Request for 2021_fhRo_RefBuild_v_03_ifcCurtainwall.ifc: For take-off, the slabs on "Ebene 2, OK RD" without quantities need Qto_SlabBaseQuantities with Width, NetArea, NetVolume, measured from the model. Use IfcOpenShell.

First a look at what the model holds.

```python
import ifcopenshell
import ifcopenshell.util.element
import ifcopenshell.util.unit

model = ifcopenshell.open("2021_fhRo_RefBuild_v_03_ifcCurtainwall.ifc")
print(model.schema)
for unit_type in ("LENGTHUNIT", "AREAUNIT", "VOLUMEUNIT"):
    print(unit_type, ifcopenshell.util.unit.calculate_unit_scale(model, unit_type))
storey = next(s for s in model.by_type("IfcBuildingStorey") if s.Name == "Ebene 2, OK RD")
slabs = [e for e in ifcopenshell.util.element.get_decomposition(storey) if e.is_a("IfcSlab")]
for e in sorted(slabs, key=lambda e: e.id()):
    print(e.id(), e.is_a(), e.Name, list(ifcopenshell.util.element.get_psets(e, qtos_only=True)), sep=" | ")
```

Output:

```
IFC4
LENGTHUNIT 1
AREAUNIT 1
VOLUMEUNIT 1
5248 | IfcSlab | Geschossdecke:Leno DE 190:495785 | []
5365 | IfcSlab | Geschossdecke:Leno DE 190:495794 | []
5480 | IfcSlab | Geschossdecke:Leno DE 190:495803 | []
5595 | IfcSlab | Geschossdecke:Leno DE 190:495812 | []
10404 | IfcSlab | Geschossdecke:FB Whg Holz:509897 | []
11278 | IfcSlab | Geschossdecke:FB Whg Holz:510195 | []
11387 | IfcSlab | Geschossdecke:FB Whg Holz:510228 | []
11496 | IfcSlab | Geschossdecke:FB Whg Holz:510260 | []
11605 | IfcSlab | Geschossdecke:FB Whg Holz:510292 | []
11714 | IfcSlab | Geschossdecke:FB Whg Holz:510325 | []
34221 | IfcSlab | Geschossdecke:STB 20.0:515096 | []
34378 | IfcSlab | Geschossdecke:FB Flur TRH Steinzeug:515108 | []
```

```python
import ifcopenshell
import ifcopenshell.api.pset
import ifcopenshell.geom
import ifcopenshell.util.element
import ifcopenshell.util.shape
import ifcopenshell.util.unit

model = ifcopenshell.open("2021_fhRo_RefBuild_v_03_ifcCurtainwall.ifc")
unit_scale = ifcopenshell.util.unit.calculate_unit_scale(model)
area_scale = ifcopenshell.util.unit.calculate_unit_scale(model, "AREAUNIT")
volume_scale = ifcopenshell.util.unit.calculate_unit_scale(model, "VOLUMEUNIT")
settings = ifcopenshell.geom.settings()

storey = next(s for s in model.by_type("IfcBuildingStorey") if s.Name == "Ebene 2, OK RD")
slabs = [e for e in ifcopenshell.util.element.get_decomposition(storey) if e.is_a("IfcSlab")]

for e in sorted(slabs, key=lambda e: e.id()):
    if ifcopenshell.util.element.get_psets(e, qtos_only=True, should_inherit=False):
        continue
    # Geometry comes back in metres, in the element's own axes.
    shape = ifcopenshell.geom.create_shape(settings, e)
    values = {
        "Width": ifcopenshell.util.shape.get_z(shape.geometry) / unit_scale,
        "NetArea": ifcopenshell.util.shape.get_footprint_area(shape.geometry) / area_scale,
        "NetVolume": ifcopenshell.util.shape.get_volume(shape.geometry) / volume_scale,
    }
    qto = ifcopenshell.api.pset.add_qto(model, product=e, name="Qto_SlabBaseQuantities")
    ifcopenshell.api.pset.edit_qto(model, qto=qto, properties=values)
    print(e.id(), {k: round(v, 3) for k, v in values.items()})

model.write("2021_fhRo_RefBuild_v_03_ifcCurtainwall_v2.ifc")
```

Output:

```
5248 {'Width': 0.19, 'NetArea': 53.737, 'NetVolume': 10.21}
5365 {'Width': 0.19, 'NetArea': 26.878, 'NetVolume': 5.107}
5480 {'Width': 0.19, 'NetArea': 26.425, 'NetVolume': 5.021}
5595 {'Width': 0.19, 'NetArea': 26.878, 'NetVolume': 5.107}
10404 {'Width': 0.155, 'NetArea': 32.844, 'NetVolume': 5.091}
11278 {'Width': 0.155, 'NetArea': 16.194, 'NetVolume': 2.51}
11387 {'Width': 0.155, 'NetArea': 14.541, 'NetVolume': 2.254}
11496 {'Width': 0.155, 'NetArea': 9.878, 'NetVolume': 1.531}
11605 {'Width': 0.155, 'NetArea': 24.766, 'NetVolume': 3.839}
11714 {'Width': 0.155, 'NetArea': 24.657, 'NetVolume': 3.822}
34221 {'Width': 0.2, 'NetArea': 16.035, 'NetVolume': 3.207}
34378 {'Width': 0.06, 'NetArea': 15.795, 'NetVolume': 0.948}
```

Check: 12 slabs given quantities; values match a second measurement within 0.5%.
